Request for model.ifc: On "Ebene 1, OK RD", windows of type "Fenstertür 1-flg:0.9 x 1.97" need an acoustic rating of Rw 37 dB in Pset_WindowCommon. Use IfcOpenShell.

First a look at what the model holds.

```python
import ifcopenshell
import ifcopenshell.util.element

model = ifcopenshell.open("model.ifc")
print(model.schema)
storey = next(s for s in model.by_type("IfcBuildingStorey") if s.Name == "Ebene 1, OK RD")
windows = [e for e in ifcopenshell.util.element.get_decomposition(storey) if e.is_a("IfcWindow")]
seen = {}
for e in windows:
    element_type = ifcopenshell.util.element.get_type(e)
    key = (element_type.Name if element_type != e and element_type else None, ifcopenshell.util.element.get_pset(e, "Pset_WindowCommon", "AcousticRating"))
    seen[key] = seen.get(key, 0) + 1
for (name, value), count in sorted(seen.items(), key=str):
    print(count, "x", name, "|", value)
```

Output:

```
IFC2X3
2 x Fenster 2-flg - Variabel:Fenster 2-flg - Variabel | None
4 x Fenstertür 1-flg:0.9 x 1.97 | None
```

```python
import ifcopenshell
import ifcopenshell.api.pset
import ifcopenshell.util.element

model = ifcopenshell.open("model.ifc")

storey = next(s for s in model.by_type("IfcBuildingStorey") if s.Name == "Ebene 1, OK RD")
windows = [e for e in ifcopenshell.util.element.get_decomposition(storey) if e.is_a("IfcWindow")]

count = 0
for e in windows:
    element_type = ifcopenshell.util.element.get_type(e)
    if element_type in (None, e) or element_type.Name != "Fenstertür 1-flg:0.9 x 1.97":
        continue
    # add_pset returns the element's existing set when there is one.
    pset = ifcopenshell.api.pset.add_pset(model, product=e, name="Pset_WindowCommon")
    ifcopenshell.api.pset.edit_pset(model, pset=pset, properties={"AcousticRating": "Rw 37 dB"})
    count += 1

print(count, "windows updated")

model.write("model_v2.ifc")
```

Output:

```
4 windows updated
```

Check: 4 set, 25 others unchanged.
